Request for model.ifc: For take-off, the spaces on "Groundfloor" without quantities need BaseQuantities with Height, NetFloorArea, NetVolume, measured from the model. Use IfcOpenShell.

First a look at what the model holds.

```python
import ifcopenshell
import ifcopenshell.util.element
import ifcopenshell.util.unit

model = ifcopenshell.open("model.ifc")
print(model.schema)
for unit_type in ("LENGTHUNIT", "AREAUNIT", "VOLUMEUNIT"):
    print(unit_type, ifcopenshell.util.unit.calculate_unit_scale(model, unit_type))
storey = next(s for s in model.by_type("IfcBuildingStorey") if s.Name == "Groundfloor")
spaces = [e for e in ifcopenshell.util.element.get_decomposition(storey) if e.is_a("IfcSpace")]
for e in sorted(spaces, key=lambda e: e.id()):
    print(e.id(), e.is_a(), e.Name, list(ifcopenshell.util.element.get_psets(e, qtos_only=True)), sep=" | ")
```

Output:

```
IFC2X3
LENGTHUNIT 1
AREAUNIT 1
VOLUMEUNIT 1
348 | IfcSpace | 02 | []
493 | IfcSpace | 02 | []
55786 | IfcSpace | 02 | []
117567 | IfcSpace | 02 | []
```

```python
import ifcopenshell
import ifcopenshell.api.pset
import ifcopenshell.geom
import ifcopenshell.util.element
import ifcopenshell.util.shape
import ifcopenshell.util.unit

model = ifcopenshell.open("model.ifc")
unit_scale = ifcopenshell.util.unit.calculate_unit_scale(model)
area_scale = ifcopenshell.util.unit.calculate_unit_scale(model, "AREAUNIT")
volume_scale = ifcopenshell.util.unit.calculate_unit_scale(model, "VOLUMEUNIT")
settings = ifcopenshell.geom.settings()

storey = next(s for s in model.by_type("IfcBuildingStorey") if s.Name == "Groundfloor")
spaces = [e for e in ifcopenshell.util.element.get_decomposition(storey) if e.is_a("IfcSpace")]

for e in sorted(spaces, key=lambda e: e.id()):
    if ifcopenshell.util.element.get_psets(e, qtos_only=True, should_inherit=False):
        continue
    # Geometry comes back in metres, in the element's own axes.
    shape = ifcopenshell.geom.create_shape(settings, e)
    values = {
        "Height": ifcopenshell.util.shape.get_z(shape.geometry) / unit_scale,
        "NetFloorArea": ifcopenshell.util.shape.get_footprint_area(shape.geometry) / area_scale,
        "NetVolume": ifcopenshell.util.shape.get_volume(shape.geometry) / volume_scale,
    }
    qto = ifcopenshell.api.pset.add_qto(model, product=e, name="BaseQuantities")
    ifcopenshell.api.pset.edit_qto(model, qto=qto, properties=values)
    print(e.id(), {k: round(v, 3) for k, v in values.items()})

model.write("model_edited.ifc")
```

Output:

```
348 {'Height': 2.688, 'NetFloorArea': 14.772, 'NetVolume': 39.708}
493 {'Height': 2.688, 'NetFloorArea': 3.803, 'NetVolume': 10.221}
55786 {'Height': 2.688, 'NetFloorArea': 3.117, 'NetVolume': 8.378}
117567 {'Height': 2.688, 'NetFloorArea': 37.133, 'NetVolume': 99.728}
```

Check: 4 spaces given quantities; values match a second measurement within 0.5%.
